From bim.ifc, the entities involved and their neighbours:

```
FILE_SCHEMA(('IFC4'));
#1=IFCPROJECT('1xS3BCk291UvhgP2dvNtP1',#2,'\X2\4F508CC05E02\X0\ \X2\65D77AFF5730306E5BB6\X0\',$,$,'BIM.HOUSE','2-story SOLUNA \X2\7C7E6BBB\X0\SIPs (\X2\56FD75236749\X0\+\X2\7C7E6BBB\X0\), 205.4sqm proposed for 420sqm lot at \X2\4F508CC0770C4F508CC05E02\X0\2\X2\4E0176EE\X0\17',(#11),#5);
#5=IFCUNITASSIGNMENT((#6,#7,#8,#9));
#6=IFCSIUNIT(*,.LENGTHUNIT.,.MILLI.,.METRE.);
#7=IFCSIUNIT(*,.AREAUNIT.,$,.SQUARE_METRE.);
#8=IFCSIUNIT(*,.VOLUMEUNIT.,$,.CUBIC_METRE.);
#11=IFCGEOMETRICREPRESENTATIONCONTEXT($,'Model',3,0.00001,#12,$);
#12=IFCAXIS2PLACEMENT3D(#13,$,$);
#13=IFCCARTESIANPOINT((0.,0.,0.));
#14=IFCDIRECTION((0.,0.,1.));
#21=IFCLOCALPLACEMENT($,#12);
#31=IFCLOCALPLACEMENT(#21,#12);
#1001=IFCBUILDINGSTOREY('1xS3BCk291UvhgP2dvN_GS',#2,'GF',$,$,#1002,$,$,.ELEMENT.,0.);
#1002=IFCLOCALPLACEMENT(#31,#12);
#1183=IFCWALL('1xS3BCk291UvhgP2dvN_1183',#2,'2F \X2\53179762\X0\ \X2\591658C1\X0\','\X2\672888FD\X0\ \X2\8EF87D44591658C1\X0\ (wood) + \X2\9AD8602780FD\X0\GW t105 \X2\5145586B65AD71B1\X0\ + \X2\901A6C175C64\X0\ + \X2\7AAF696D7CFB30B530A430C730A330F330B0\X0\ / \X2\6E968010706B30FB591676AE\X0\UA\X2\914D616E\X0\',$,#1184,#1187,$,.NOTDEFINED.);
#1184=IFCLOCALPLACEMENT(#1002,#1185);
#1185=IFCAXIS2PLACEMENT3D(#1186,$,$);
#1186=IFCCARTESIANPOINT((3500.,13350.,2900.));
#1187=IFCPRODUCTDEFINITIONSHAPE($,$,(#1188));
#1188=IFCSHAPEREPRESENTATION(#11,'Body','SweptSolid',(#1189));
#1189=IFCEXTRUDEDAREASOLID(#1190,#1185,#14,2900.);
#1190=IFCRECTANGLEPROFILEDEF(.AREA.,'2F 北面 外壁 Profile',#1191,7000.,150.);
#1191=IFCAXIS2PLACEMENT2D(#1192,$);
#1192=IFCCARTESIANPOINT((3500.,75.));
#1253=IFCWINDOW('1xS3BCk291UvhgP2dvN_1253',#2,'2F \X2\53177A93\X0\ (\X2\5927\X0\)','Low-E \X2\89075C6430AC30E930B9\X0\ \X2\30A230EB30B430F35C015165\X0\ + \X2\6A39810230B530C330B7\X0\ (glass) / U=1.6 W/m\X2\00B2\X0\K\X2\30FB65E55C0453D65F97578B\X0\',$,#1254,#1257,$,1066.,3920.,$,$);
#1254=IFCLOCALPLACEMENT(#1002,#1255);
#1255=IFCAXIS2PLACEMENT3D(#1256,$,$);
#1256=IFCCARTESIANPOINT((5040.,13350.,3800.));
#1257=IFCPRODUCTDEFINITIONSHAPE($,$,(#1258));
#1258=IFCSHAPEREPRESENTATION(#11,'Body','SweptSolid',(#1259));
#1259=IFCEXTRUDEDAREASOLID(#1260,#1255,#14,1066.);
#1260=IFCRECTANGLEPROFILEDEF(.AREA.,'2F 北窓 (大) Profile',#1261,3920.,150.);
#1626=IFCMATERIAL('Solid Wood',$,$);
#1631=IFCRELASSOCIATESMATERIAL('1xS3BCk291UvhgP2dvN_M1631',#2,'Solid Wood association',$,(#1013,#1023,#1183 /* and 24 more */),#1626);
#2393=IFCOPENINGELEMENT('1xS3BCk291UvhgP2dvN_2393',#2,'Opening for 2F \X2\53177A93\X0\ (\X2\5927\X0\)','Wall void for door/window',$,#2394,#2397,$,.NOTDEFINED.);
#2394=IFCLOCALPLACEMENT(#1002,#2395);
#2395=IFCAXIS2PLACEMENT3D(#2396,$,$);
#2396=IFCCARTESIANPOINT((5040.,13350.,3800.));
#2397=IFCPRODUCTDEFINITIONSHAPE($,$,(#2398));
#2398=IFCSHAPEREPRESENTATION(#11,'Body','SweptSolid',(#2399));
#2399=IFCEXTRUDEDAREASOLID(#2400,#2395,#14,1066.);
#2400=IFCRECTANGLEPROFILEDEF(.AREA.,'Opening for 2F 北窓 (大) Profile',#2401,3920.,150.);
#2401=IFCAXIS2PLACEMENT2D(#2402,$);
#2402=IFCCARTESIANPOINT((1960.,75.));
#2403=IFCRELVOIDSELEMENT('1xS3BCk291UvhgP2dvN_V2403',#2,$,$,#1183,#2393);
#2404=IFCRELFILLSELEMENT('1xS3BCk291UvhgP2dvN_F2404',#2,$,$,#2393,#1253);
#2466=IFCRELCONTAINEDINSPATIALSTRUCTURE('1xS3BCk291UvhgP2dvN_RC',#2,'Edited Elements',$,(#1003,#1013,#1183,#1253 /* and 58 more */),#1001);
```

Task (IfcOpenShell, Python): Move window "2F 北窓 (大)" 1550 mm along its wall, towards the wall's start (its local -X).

```python
import ifcopenshell
import ifcopenshell.api.geometry
import ifcopenshell.util.placement
import ifcopenshell.util.unit

model = ifcopenshell.open("bim.ifc")
unit_scale = ifcopenshell.util.unit.calculate_unit_scale(model)

window = model.by_guid("1xS3BCk291UvhgP2dvN_1253")
opening = window.FillsVoids[0].RelatingOpeningElement
wall = opening.VoidsElements[0].RelatingBuildingElement

wall_matrix = ifcopenshell.util.placement.get_local_placement(wall.ObjectPlacement)
shift = wall_matrix[:3, 0] * -1.55 / unit_scale
before = ifcopenshell.util.placement.get_local_placement(window.ObjectPlacement)[:3, 3].copy()

# The window is not placed relative to its opening, so move both.
for product in (opening, window):
    matrix = ifcopenshell.util.placement.get_local_placement(product.ObjectPlacement)
    matrix[:3, 3] += shift
    ifcopenshell.api.geometry.edit_object_placement(model, product=product, matrix=matrix, is_si=False)

after = ifcopenshell.util.placement.get_local_placement(window.ObjectPlacement)[:3, 3]
print("window moved by", (after - before).round(3) + 0.0)

model.write("bim_edited.ifc")
```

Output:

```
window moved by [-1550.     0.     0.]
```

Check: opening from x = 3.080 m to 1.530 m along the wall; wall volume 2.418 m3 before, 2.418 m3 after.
